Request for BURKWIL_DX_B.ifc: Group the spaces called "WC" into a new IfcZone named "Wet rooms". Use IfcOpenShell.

First a look at what the model holds.

```python
import ifcopenshell

model = ifcopenshell.open("BURKWIL_DX_B.ifc")
print(model.schema)
seen = {}
for space in model.by_type("IfcSpace"):
    seen[space.LongName] = seen.get(space.LongName, 0) + 1
for name, count in sorted(seen.items(), key=str):
    print(count, "x", name)
print("zones:", [z.Name for z in model.by_type("IfcZone")][:20])
```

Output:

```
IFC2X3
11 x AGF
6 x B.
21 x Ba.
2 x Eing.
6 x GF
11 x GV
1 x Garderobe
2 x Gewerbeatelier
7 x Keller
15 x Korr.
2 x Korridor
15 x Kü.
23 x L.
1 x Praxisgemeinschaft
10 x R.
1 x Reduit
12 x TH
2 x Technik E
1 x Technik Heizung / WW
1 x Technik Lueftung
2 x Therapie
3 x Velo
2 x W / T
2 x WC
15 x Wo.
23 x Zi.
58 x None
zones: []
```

```python
import ifcopenshell
import ifcopenshell.api.group
import ifcopenshell.api.root

model = ifcopenshell.open("BURKWIL_DX_B.ifc")

names = {"WC"}
spaces = [s for s in model.by_type("IfcSpace") if s.LongName in names]

zone = ifcopenshell.api.root.create_entity(model, ifc_class="IfcZone", name="Wet rooms")
ifcopenshell.api.group.assign_group(model, products=spaces, group=zone)
print(len(spaces), "spaces in", zone.Name)

model.write("BURKWIL_DX_B_edited.ifc")
```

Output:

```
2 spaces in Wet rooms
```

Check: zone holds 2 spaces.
